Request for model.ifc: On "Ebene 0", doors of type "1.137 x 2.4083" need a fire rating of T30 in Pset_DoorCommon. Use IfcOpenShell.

First a look at what the model holds.

```python
import ifcopenshell
import ifcopenshell.util.element

model = ifcopenshell.open("model.ifc")
print(model.schema)
storey = next(s for s in model.by_type("IfcBuildingStorey") if s.Name == "Ebene 0")
doors = [e for e in ifcopenshell.util.element.get_decomposition(storey) if e.is_a("IfcDoor")]
seen = {}
for e in doors:
    element_type = ifcopenshell.util.element.get_type(e)
    key = (element_type.Name if element_type != e and element_type else None, ifcopenshell.util.element.get_pset(e, "Pset_DoorCommon", "FireRating"))
    seen[key] = seen.get(key, 0) + 1
for (name, value), count in sorted(seen.items(), key=str):
    print(count, "x", name, "|", value)
```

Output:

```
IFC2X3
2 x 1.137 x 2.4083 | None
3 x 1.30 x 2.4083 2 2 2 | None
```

```python
import ifcopenshell
import ifcopenshell.api.pset
import ifcopenshell.util.element

model = ifcopenshell.open("model.ifc")

storey = next(s for s in model.by_type("IfcBuildingStorey") if s.Name == "Ebene 0")
doors = [e for e in ifcopenshell.util.element.get_decomposition(storey) if e.is_a("IfcDoor")]

count = 0
for e in doors:
    element_type = ifcopenshell.util.element.get_type(e)
    if element_type in (None, e) or element_type.Name != "1.137 x 2.4083":
        continue
    # add_pset returns the element's existing set when there is one.
    pset = ifcopenshell.api.pset.add_pset(model, product=e, name="Pset_DoorCommon")
    ifcopenshell.api.pset.edit_pset(model, pset=pset, properties={"FireRating": "T30"})
    count += 1

print(count, "doors updated")

model.write("model_v2.ifc")
```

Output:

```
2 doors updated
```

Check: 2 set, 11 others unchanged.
